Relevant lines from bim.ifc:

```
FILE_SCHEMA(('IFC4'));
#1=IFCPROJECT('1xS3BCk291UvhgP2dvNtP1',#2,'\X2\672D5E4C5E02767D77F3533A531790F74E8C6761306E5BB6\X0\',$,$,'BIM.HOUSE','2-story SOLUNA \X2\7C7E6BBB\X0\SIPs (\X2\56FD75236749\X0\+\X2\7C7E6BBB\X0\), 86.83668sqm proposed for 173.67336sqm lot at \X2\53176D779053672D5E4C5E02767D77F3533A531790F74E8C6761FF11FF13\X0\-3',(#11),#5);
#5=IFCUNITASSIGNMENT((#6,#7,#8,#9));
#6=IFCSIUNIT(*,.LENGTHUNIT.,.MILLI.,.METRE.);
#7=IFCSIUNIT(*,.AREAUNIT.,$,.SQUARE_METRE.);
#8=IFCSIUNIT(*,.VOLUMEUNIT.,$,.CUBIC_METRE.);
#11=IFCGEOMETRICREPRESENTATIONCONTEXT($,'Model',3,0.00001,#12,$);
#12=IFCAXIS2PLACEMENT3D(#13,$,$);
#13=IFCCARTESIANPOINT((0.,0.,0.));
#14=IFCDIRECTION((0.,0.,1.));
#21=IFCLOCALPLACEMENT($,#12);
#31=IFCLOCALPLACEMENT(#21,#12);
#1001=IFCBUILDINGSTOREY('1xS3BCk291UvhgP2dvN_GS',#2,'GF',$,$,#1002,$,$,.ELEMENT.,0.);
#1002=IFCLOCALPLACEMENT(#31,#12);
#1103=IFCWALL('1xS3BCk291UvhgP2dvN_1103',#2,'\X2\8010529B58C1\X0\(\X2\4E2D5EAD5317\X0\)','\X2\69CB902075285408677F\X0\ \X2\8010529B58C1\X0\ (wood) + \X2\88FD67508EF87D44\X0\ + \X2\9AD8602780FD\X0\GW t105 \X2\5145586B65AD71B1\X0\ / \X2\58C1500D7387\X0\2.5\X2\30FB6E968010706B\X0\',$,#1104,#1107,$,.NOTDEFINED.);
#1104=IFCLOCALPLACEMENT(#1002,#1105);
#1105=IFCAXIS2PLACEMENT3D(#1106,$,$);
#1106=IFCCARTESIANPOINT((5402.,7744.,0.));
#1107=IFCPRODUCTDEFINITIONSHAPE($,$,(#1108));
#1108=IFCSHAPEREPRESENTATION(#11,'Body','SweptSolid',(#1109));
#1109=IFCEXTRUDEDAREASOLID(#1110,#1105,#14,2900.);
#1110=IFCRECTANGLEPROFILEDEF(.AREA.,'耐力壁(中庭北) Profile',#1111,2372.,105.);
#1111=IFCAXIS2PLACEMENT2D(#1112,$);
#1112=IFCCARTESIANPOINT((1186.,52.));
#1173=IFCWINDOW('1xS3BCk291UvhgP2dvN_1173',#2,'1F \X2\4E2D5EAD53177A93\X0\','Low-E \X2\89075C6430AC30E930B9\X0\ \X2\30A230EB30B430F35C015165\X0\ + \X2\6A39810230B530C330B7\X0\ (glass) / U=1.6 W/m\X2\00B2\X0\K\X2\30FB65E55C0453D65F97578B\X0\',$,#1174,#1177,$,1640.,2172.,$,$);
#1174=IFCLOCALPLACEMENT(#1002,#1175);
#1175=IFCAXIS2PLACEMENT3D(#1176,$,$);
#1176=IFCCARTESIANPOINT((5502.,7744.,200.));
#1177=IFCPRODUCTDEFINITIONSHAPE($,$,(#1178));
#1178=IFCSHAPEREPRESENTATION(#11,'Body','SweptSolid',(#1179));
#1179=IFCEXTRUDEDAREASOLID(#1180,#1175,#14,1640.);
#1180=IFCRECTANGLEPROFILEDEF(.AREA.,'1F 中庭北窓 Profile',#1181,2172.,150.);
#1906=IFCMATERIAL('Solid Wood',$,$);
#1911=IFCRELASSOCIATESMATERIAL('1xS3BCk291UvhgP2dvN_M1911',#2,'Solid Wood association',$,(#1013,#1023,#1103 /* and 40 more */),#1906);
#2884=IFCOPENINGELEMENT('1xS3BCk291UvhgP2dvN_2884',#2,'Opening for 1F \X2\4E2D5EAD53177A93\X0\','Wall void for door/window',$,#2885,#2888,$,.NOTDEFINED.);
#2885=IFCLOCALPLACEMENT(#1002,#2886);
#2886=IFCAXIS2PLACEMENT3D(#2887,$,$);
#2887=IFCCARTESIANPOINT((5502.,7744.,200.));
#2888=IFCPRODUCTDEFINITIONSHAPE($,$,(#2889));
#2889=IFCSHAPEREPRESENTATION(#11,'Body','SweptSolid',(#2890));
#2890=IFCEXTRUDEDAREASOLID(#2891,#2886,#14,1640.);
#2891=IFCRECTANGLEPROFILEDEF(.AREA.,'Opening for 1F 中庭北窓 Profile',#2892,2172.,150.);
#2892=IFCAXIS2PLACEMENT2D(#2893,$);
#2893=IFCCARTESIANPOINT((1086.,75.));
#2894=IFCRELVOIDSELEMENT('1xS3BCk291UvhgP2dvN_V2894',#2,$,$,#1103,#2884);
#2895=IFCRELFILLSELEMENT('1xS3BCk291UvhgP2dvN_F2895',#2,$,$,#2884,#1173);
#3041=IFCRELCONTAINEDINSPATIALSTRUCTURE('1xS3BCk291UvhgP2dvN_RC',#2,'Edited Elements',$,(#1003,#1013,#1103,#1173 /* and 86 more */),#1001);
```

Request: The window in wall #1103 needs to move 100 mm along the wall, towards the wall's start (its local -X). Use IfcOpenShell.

```python
import ifcopenshell
import ifcopenshell.api.geometry
import ifcopenshell.util.placement
import ifcopenshell.util.unit

model = ifcopenshell.open("bim.ifc")
unit_scale = ifcopenshell.util.unit.calculate_unit_scale(model)

window = model.by_guid("1xS3BCk291UvhgP2dvN_1173")
opening = window.FillsVoids[0].RelatingOpeningElement
wall = opening.VoidsElements[0].RelatingBuildingElement

wall_matrix = ifcopenshell.util.placement.get_local_placement(wall.ObjectPlacement)
shift = wall_matrix[:3, 0] * -0.1 / unit_scale
before = ifcopenshell.util.placement.get_local_placement(window.ObjectPlacement)[:3, 3].copy()

# The window is not placed relative to its opening, so move both.
for product in (opening, window):
    matrix = ifcopenshell.util.placement.get_local_placement(product.ObjectPlacement)
    matrix[:3, 3] += shift
    ifcopenshell.api.geometry.edit_object_placement(model, product=product, matrix=matrix, is_si=False)

after = ifcopenshell.util.placement.get_local_placement(window.ObjectPlacement)[:3, 3]
print("window moved by", (after - before).round(3) + 0.0)

model.write("bim_updated.ifc")
```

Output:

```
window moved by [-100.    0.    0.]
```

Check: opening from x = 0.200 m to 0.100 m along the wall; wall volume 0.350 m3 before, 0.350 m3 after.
